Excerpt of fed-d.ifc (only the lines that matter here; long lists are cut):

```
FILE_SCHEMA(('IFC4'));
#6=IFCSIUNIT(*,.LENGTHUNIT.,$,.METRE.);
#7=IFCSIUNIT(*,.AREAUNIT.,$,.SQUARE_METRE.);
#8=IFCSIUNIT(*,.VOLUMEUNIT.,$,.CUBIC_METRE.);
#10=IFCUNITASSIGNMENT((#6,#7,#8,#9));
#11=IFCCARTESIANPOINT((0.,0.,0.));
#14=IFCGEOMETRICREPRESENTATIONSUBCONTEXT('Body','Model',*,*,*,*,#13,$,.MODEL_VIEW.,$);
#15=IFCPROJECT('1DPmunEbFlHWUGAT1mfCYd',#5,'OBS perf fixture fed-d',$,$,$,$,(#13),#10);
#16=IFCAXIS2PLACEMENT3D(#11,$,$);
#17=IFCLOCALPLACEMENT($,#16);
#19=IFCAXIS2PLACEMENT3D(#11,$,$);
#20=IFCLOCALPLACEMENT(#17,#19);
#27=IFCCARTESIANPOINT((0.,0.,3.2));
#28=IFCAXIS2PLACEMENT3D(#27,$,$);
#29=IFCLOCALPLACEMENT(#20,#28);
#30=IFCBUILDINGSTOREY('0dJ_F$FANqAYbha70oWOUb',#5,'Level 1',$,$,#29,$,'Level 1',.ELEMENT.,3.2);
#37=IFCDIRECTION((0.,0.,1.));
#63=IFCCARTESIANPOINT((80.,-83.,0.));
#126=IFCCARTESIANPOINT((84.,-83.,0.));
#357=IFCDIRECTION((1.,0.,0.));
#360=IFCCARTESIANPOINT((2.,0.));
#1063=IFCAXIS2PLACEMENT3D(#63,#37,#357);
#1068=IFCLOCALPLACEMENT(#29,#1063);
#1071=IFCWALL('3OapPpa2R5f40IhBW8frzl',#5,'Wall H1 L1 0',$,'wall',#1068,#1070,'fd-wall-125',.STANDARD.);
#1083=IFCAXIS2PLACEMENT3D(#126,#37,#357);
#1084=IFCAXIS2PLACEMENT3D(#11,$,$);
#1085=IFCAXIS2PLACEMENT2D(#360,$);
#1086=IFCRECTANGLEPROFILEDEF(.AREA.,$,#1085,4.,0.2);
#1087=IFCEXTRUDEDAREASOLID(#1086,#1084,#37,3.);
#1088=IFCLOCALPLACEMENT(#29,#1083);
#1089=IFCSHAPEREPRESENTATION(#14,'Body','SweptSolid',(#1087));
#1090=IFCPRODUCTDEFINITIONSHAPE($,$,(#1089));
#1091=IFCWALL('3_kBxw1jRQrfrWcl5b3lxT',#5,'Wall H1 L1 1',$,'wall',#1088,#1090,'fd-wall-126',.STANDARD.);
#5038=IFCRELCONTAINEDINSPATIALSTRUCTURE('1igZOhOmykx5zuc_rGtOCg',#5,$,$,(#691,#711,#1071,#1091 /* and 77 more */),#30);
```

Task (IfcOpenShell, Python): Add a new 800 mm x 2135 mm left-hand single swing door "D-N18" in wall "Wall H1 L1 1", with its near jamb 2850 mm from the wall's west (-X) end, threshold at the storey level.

```python
import numpy as np
import ifcopenshell
import ifcopenshell.api.feature
import ifcopenshell.api.geometry
import ifcopenshell.api.root
import ifcopenshell.api.spatial
import ifcopenshell.geom
import ifcopenshell.util.element
import ifcopenshell.util.placement
import ifcopenshell.util.representation
import ifcopenshell.util.shape
import ifcopenshell.util.unit

model = ifcopenshell.open("fed-d.ifc")
unit_scale = ifcopenshell.util.unit.calculate_unit_scale(model)
settings = ifcopenshell.geom.settings()


def volume(element):
    """Net volume in cubic metres, openings subtracted."""
    shape = ifcopenshell.geom.create_shape(settings, element)
    return ifcopenshell.util.shape.get_volume(shape.geometry)


wall = model.by_id(1091)
storey = ifcopenshell.util.element.get_container(wall, ifc_class="IfcBuildingStorey")
context = ifcopenshell.util.representation.get_context(model, "Model", "Body", "MODEL_VIEW")
before = volume(wall)

width, height, from_end, sill = 0.8, 2.135, 2.85, 0.0  # metres

# The wall runs along its own X axis, and the end named is its -X end.
wall_shape = ifcopenshell.geom.create_shape(settings, wall)
x, y, z = ifcopenshell.util.shape.get_vertices(wall_shape.geometry).T
start = x.min() + from_end
face, thickness = float(y.min()), float(y.max() - y.min())
wall_matrix = ifcopenshell.util.placement.get_local_placement(wall.ObjectPlacement)
level = ifcopenshell.util.placement.get_local_placement(storey.ObjectPlacement)[2, 3]


def in_wall(x, y):
    """Placement at x, y metres in the wall's axes, at sill height."""
    matrix = wall_matrix.copy()
    matrix[:, 3] = wall_matrix @ np.array([x / unit_scale, y / unit_scale, 0.0, 1.0])
    matrix[2, 3] = level + sill / unit_scale
    return matrix


# Opening: a box that overshoots both wall faces by 50 mm.
opening = ifcopenshell.api.root.create_entity(model, ifc_class="IfcOpeningElement", predefined_type="OPENING")
box = ifcopenshell.api.geometry.add_wall_representation(
    model, context=context, length=width, height=height, thickness=thickness + 0.1
)
ifcopenshell.api.geometry.assign_representation(model, product=opening, representation=box)
ifcopenshell.api.geometry.edit_object_placement(model, product=opening, matrix=in_wall(start, face - 0.05), is_si=False)
ifcopenshell.api.feature.add_feature(model, feature=opening, element=wall)

door = ifcopenshell.api.root.create_entity(model, ifc_class="IfcDoor", name="D-N18", predefined_type="DOOR")
door.OverallWidth, door.OverallHeight = width / unit_scale, height / unit_scale
door.OperationType = "SINGLE_SWING_LEFT"
body = ifcopenshell.api.geometry.add_door_representation(
    model,
    context=context,
    overall_width=door.OverallWidth,
    overall_height=door.OverallHeight,
    operation_type="SINGLE_SWING_LEFT",
    lining_properties={"LiningDepth": thickness / unit_scale, "ThresholdDepth": thickness / unit_scale},
)
ifcopenshell.api.geometry.assign_representation(model, product=door, representation=body)
ifcopenshell.api.spatial.assign_container(model, products=[door], relating_structure=storey)
ifcopenshell.api.feature.add_filling(model, opening=opening, element=door)

# The lining spans the wall, so the door starts at the wall face.
ifcopenshell.api.geometry.edit_object_placement(model, product=door, matrix=in_wall(start, face), is_si=False)

after = volume(wall)

print(f"wall volume {before:.3f} -> {after:.3f} m3")

model.write("fed-d-out.ifc")
```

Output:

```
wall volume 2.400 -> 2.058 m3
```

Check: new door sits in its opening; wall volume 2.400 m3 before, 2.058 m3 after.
